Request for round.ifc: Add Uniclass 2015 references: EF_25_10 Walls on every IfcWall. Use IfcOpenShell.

First a look at what the model holds.

```python
import ifcopenshell

model = ifcopenshell.open("round.ifc")
print(model.schema)
print("classifications:", [c.Name for c in model.by_type("IfcClassification")])
for ifc_class in ("IfcDoor", "IfcRoof", "IfcStair", "IfcWall", "IfcWindow"):
    print(ifc_class, len(model.by_type(ifc_class)))
```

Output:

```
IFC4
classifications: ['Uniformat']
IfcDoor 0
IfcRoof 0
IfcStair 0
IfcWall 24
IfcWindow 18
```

```python
import ifcopenshell
import ifcopenshell.api.classification

model = ifcopenshell.open("round.ifc")

system = ifcopenshell.api.classification.add_classification(model, classification="Uniclass 2015")

codes = {
    "IfcWall": ("EF_25_10", "Walls"),
}
for ifc_class, (code, name) in codes.items():
    products = model.by_type(ifc_class)
    ifcopenshell.api.classification.add_reference(
        model, products=products, classification=system, identification=code, name=name
    )
    print(code, len(products))

model.write("round_edited.ifc")
```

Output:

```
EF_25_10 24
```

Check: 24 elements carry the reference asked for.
